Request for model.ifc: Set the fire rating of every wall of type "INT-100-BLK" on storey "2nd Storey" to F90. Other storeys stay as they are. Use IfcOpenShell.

First a look at what the model holds.

```python
import ifcopenshell
import ifcopenshell.util.element

model = ifcopenshell.open("model.ifc")
print(model.schema)
storey = next(s for s in model.by_type("IfcBuildingStorey") if s.Name == "2nd Storey")
walls = [e for e in ifcopenshell.util.element.get_decomposition(storey) if e.is_a("IfcWall")]
seen = {}
for e in walls:
    element_type = ifcopenshell.util.element.get_type(e)
    key = (element_type.Name if element_type != e and element_type else None, ifcopenshell.util.element.get_pset(e, "Pset_WallCommon", "FireRating"))
    seen[key] = seen.get(key, 0) + 1
for (name, value), count in sorted(seen.items(), key=str):
    print(count, "x", name, "|", value)
```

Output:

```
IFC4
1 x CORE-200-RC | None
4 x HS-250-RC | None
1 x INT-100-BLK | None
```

```python
import ifcopenshell
import ifcopenshell.api.pset
import ifcopenshell.util.element

model = ifcopenshell.open("model.ifc")

storey = next(s for s in model.by_type("IfcBuildingStorey") if s.Name == "2nd Storey")
walls = [e for e in ifcopenshell.util.element.get_decomposition(storey) if e.is_a("IfcWall")]

count = 0
for e in walls:
    element_type = ifcopenshell.util.element.get_type(e)
    if element_type in (None, e) or element_type.Name != "INT-100-BLK":
        continue
    # add_pset returns the element's existing set when there is one.
    pset = ifcopenshell.api.pset.add_pset(model, product=e, name="Pset_WallCommon")
    ifcopenshell.api.pset.edit_pset(model, pset=pset, properties={"FireRating": "F90"})
    count += 1

print(count, "walls updated")

model.write("model-out.ifc")
```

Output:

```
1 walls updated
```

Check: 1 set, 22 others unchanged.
